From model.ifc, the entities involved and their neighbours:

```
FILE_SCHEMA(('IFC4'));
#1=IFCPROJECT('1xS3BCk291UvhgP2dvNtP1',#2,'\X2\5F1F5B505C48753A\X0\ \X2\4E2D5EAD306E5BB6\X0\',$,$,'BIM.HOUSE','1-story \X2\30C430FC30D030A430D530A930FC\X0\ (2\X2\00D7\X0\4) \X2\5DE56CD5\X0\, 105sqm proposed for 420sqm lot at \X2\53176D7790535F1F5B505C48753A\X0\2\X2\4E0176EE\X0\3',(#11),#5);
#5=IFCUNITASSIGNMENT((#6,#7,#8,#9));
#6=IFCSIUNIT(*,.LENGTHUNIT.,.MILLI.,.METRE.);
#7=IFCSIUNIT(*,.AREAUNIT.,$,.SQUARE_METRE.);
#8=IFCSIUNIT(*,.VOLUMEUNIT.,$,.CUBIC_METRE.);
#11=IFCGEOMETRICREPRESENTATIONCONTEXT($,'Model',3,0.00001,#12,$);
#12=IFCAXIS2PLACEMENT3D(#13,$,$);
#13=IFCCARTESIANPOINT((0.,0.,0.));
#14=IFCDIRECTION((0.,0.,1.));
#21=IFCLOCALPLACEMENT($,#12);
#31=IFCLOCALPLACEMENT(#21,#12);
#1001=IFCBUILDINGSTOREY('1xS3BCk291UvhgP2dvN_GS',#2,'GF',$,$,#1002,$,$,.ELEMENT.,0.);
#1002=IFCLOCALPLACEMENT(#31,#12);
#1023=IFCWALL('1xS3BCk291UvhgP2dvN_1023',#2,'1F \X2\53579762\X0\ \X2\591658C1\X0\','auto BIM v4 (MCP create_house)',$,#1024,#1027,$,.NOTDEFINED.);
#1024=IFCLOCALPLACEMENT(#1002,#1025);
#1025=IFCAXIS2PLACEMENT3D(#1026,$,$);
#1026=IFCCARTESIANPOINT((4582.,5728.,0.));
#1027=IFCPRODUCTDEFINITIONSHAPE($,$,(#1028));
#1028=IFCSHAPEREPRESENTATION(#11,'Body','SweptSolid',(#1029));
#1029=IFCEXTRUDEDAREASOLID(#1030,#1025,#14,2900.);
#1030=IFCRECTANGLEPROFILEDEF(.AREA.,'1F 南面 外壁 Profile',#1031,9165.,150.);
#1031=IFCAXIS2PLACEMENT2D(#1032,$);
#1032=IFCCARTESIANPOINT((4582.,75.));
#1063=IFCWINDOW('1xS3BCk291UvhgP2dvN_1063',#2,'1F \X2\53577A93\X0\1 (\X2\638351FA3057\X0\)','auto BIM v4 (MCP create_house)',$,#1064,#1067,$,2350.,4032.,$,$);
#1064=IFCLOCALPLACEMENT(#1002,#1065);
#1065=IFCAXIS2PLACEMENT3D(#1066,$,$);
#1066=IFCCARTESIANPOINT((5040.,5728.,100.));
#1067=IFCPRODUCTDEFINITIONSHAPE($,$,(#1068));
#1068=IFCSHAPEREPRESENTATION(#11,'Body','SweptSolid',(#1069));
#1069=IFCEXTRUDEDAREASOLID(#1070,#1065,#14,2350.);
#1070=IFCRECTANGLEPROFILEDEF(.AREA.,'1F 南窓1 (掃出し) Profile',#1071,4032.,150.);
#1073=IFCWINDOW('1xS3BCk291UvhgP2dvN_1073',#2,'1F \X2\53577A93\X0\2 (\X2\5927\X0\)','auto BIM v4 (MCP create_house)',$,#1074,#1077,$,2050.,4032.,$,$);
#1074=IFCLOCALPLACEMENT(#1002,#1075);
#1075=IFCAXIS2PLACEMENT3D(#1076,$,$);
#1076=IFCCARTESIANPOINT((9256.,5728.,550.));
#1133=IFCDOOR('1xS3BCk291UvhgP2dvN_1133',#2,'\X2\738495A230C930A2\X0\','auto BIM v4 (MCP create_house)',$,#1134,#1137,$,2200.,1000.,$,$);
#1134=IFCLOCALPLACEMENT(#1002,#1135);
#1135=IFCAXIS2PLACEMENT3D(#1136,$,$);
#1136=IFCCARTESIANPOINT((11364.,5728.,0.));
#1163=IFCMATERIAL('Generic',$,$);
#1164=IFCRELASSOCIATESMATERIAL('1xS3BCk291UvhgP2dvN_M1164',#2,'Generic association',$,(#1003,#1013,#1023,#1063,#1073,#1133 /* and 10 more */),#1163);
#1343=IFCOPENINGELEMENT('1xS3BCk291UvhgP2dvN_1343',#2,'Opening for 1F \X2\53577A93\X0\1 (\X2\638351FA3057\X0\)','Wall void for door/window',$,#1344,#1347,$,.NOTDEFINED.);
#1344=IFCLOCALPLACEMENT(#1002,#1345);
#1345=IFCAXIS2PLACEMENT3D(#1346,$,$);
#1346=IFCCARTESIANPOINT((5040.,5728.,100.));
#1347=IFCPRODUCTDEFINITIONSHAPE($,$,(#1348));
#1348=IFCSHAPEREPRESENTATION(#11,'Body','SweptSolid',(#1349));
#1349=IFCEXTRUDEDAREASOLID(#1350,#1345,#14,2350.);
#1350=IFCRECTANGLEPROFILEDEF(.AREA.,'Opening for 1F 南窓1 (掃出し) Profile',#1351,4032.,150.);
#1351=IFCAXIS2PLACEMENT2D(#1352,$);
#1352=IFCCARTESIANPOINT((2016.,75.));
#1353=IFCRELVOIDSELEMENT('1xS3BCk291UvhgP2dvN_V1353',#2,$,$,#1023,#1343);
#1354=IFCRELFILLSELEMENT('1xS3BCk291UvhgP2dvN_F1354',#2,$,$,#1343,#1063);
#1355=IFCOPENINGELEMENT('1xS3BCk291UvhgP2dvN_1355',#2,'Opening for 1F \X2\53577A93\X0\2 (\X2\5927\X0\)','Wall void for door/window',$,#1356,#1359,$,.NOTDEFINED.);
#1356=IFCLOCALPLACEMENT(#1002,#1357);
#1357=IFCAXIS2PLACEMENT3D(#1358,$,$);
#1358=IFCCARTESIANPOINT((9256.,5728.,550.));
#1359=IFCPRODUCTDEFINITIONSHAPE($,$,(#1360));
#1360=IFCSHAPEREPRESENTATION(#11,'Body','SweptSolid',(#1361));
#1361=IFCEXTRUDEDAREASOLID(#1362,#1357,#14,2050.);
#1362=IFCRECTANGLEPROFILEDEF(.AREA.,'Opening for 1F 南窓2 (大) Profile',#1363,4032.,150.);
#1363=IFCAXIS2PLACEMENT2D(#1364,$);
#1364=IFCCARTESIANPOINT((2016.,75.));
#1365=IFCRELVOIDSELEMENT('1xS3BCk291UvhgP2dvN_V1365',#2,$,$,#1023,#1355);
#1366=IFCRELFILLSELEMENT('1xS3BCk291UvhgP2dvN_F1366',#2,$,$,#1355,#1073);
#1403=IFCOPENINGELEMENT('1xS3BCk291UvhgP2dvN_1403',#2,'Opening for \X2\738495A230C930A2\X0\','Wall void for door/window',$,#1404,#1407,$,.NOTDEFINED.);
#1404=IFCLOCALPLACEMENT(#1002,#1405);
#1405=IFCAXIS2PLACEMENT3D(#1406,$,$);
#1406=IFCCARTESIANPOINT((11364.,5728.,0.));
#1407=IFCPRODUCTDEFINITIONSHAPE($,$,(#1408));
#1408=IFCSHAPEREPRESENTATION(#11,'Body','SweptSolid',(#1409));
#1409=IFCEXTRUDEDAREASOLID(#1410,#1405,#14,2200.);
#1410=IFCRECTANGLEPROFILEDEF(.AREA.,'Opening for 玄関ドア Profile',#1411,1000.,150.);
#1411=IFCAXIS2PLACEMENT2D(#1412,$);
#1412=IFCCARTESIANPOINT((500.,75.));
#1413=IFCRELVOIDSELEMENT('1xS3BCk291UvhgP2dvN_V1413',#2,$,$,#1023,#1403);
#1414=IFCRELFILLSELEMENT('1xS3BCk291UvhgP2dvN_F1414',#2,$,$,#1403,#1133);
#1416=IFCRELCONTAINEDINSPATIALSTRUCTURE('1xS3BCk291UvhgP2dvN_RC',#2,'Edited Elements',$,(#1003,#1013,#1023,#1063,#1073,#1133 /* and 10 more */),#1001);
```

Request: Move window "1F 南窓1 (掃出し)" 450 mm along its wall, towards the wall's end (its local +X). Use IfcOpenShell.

```python
import ifcopenshell
import ifcopenshell.api.geometry
import ifcopenshell.util.placement

model = ifcopenshell.open("model.ifc")

window = model.by_guid("1xS3BCk291UvhgP2dvN_1063")
opening = window.FillsVoids[0].RelatingOpeningElement
wall = opening.VoidsElements[0].RelatingBuildingElement

wall_matrix = ifcopenshell.util.placement.get_local_placement(wall.ObjectPlacement)
shift = wall_matrix[:3, 0] * 450.0
before = ifcopenshell.util.placement.get_local_placement(window.ObjectPlacement)[:3, 3].copy()

# The window is not placed relative to its opening, so move both.
for product in (opening, window):
    matrix = ifcopenshell.util.placement.get_local_placement(product.ObjectPlacement)
    matrix[:3, 3] += shift
    ifcopenshell.api.geometry.edit_object_placement(model, product=product, matrix=matrix, is_si=False)

after = ifcopenshell.util.placement.get_local_placement(window.ObjectPlacement)[:3, 3]
print("window moved by", (after - before).round(3) + 0.0)

model.write("model_v2.ifc")
```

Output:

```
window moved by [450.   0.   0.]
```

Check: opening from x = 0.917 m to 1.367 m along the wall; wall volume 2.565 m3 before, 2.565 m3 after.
